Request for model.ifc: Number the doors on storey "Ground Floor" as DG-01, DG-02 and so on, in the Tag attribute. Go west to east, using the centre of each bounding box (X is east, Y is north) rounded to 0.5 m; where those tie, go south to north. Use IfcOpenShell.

First a look at what the model holds.

```python
import ifcopenshell
import ifcopenshell.util.element
import ifcopenshell.util.placement

model = ifcopenshell.open("model.ifc")
print(model.schema)
storey = next(s for s in model.by_type("IfcBuildingStorey") if s.Name == "Ground Floor")
doors = [e for e in ifcopenshell.util.element.get_decomposition(storey) if e.is_a("IfcDoor")]
for e in sorted(doors, key=lambda e: e.id()):
    origin = ifcopenshell.util.placement.get_local_placement(e.ObjectPlacement)[:3, 3]
    print(e.id(), e.Tag, e.Name, origin.round(2) + 0.0, sep=" | ")
```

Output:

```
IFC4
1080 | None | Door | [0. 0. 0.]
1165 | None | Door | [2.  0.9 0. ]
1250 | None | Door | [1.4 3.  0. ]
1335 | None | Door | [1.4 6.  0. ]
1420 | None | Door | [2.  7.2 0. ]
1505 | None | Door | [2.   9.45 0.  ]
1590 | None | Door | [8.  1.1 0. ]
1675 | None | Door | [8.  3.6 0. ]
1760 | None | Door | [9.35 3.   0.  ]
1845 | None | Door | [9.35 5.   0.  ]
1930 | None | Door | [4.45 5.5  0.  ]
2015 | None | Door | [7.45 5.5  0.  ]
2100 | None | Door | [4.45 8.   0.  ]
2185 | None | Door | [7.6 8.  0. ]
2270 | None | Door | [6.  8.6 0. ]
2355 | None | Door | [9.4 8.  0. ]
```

```python
import ifcopenshell
import ifcopenshell.geom
import ifcopenshell.util.element
import ifcopenshell.util.shape

model = ifcopenshell.open("model.ifc")
settings = ifcopenshell.geom.settings()
settings.set("use-world-coords", True)


def centre(element):
    shape = ifcopenshell.geom.create_shape(settings, element)
    return ifcopenshell.util.shape.get_bbox_centroid(shape.geometry)


storey = next(s for s in model.by_type("IfcBuildingStorey") if s.Name == "Ground Floor")
doors = [e for e in ifcopenshell.util.element.get_decomposition(storey) if e.is_a("IfcDoor")]

# Insertion points can sit at a corner or the storey origin, so sort by the geometry (in metres).
centres = {e: centre(e) for e in doors}
doors.sort(key=lambda e: (round(centres[e][0] / 0.5), centres[e][1]))

for i, e in enumerate(doors, start=1):
    number = f"DG-{i:02d}"
    e.Tag = number
    print(e.id(), number)

model.write("model_updated.ifc")
```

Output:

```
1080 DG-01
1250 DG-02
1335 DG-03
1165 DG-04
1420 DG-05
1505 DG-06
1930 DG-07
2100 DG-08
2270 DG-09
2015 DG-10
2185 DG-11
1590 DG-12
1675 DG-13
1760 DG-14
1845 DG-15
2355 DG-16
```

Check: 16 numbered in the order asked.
